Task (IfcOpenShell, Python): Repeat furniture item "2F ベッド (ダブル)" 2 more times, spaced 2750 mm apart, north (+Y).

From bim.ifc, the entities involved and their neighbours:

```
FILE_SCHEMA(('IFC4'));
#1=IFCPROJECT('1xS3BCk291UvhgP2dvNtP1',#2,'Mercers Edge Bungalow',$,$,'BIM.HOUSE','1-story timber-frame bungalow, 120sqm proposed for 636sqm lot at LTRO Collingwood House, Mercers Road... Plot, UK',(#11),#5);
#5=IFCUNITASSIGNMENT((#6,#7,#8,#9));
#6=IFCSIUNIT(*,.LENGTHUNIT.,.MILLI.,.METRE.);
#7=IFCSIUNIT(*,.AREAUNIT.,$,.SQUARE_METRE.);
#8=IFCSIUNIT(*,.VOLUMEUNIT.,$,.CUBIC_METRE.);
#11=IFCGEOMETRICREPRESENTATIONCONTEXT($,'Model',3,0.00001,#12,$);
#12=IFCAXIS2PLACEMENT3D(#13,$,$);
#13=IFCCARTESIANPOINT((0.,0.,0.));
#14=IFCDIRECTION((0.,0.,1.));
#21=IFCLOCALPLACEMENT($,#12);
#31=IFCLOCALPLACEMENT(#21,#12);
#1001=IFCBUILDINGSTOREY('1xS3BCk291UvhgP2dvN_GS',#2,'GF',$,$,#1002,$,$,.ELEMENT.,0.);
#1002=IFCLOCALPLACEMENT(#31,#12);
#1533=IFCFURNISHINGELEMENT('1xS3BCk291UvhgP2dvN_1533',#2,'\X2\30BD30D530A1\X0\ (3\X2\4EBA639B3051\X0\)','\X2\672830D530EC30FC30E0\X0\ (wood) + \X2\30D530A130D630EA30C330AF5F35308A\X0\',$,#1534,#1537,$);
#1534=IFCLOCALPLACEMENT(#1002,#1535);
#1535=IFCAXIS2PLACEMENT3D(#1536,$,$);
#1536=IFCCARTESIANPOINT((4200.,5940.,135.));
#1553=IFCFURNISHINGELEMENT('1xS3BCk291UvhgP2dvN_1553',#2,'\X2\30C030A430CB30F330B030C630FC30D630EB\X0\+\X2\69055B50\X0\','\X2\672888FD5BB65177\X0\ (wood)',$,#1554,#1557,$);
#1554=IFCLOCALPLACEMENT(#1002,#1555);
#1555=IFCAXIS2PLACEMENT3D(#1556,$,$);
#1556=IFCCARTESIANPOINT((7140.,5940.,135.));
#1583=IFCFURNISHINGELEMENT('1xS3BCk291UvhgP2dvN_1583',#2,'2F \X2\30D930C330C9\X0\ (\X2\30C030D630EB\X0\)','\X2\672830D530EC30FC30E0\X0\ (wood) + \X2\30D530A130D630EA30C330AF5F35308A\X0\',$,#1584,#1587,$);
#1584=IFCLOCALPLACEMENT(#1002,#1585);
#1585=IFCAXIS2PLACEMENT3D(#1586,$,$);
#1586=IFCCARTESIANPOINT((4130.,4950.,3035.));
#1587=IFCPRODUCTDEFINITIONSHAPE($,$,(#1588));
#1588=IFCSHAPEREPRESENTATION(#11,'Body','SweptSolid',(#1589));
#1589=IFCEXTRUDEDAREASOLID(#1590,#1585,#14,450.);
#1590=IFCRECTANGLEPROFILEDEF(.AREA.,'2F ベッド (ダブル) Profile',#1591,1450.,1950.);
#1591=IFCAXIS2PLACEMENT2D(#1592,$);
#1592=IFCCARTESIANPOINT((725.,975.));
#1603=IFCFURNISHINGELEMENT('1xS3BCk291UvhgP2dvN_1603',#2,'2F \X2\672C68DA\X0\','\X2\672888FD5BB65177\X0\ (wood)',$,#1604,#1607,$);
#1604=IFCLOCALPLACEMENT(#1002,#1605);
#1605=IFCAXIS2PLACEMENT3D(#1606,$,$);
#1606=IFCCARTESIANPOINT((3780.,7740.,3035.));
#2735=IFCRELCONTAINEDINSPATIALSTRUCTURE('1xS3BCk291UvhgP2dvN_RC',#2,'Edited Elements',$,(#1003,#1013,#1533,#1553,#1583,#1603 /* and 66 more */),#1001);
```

```python
import numpy as np
import ifcopenshell
import ifcopenshell.api.geometry
import ifcopenshell.api.root
import ifcopenshell.util.element
import ifcopenshell.util.placement
import ifcopenshell.util.unit

model = ifcopenshell.open("bim.ifc")
unit_scale = ifcopenshell.util.unit.calculate_unit_scale(model)


def reuse_history(source, copy):
    """copy_class also copies each property set's owner history, people and application; keep the originals."""
    for rel in copy.IsDefinedBy:
        if rel.is_a("IfcRelDefinesByProperties") and (history := rel.RelatingPropertyDefinition.OwnerHistory):
            rel.RelatingPropertyDefinition.OwnerHistory = source.OwnerHistory
            ifcopenshell.util.element.remove_deep2(model, history)


source = model.by_guid("1xS3BCk291UvhgP2dvN_1583")
base = ifcopenshell.util.placement.get_local_placement(source.ObjectPlacement)
step = np.array([0.0, 1.0, 0.0]) * 2.75 / unit_scale

for i in range(1, 3):
    copy = ifcopenshell.api.root.copy_class(model, product=source)
    copy.Representation = ifcopenshell.util.element.copy_deep(
        model, source.Representation, exclude=["IfcGeometricRepresentationContext", "IfcRepresentationMap"]
    )
    reuse_history(source, copy)
    matrix = base.copy()
    matrix[:3, 3] += i * step
    print("added at", matrix[:3, 3].round(3) + 0.0)
    ifcopenshell.api.geometry.edit_object_placement(model, product=copy, matrix=matrix, is_si=False)

model.write("bim-out.ifc")
```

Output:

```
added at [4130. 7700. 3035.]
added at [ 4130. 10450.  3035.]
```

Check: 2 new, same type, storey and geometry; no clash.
